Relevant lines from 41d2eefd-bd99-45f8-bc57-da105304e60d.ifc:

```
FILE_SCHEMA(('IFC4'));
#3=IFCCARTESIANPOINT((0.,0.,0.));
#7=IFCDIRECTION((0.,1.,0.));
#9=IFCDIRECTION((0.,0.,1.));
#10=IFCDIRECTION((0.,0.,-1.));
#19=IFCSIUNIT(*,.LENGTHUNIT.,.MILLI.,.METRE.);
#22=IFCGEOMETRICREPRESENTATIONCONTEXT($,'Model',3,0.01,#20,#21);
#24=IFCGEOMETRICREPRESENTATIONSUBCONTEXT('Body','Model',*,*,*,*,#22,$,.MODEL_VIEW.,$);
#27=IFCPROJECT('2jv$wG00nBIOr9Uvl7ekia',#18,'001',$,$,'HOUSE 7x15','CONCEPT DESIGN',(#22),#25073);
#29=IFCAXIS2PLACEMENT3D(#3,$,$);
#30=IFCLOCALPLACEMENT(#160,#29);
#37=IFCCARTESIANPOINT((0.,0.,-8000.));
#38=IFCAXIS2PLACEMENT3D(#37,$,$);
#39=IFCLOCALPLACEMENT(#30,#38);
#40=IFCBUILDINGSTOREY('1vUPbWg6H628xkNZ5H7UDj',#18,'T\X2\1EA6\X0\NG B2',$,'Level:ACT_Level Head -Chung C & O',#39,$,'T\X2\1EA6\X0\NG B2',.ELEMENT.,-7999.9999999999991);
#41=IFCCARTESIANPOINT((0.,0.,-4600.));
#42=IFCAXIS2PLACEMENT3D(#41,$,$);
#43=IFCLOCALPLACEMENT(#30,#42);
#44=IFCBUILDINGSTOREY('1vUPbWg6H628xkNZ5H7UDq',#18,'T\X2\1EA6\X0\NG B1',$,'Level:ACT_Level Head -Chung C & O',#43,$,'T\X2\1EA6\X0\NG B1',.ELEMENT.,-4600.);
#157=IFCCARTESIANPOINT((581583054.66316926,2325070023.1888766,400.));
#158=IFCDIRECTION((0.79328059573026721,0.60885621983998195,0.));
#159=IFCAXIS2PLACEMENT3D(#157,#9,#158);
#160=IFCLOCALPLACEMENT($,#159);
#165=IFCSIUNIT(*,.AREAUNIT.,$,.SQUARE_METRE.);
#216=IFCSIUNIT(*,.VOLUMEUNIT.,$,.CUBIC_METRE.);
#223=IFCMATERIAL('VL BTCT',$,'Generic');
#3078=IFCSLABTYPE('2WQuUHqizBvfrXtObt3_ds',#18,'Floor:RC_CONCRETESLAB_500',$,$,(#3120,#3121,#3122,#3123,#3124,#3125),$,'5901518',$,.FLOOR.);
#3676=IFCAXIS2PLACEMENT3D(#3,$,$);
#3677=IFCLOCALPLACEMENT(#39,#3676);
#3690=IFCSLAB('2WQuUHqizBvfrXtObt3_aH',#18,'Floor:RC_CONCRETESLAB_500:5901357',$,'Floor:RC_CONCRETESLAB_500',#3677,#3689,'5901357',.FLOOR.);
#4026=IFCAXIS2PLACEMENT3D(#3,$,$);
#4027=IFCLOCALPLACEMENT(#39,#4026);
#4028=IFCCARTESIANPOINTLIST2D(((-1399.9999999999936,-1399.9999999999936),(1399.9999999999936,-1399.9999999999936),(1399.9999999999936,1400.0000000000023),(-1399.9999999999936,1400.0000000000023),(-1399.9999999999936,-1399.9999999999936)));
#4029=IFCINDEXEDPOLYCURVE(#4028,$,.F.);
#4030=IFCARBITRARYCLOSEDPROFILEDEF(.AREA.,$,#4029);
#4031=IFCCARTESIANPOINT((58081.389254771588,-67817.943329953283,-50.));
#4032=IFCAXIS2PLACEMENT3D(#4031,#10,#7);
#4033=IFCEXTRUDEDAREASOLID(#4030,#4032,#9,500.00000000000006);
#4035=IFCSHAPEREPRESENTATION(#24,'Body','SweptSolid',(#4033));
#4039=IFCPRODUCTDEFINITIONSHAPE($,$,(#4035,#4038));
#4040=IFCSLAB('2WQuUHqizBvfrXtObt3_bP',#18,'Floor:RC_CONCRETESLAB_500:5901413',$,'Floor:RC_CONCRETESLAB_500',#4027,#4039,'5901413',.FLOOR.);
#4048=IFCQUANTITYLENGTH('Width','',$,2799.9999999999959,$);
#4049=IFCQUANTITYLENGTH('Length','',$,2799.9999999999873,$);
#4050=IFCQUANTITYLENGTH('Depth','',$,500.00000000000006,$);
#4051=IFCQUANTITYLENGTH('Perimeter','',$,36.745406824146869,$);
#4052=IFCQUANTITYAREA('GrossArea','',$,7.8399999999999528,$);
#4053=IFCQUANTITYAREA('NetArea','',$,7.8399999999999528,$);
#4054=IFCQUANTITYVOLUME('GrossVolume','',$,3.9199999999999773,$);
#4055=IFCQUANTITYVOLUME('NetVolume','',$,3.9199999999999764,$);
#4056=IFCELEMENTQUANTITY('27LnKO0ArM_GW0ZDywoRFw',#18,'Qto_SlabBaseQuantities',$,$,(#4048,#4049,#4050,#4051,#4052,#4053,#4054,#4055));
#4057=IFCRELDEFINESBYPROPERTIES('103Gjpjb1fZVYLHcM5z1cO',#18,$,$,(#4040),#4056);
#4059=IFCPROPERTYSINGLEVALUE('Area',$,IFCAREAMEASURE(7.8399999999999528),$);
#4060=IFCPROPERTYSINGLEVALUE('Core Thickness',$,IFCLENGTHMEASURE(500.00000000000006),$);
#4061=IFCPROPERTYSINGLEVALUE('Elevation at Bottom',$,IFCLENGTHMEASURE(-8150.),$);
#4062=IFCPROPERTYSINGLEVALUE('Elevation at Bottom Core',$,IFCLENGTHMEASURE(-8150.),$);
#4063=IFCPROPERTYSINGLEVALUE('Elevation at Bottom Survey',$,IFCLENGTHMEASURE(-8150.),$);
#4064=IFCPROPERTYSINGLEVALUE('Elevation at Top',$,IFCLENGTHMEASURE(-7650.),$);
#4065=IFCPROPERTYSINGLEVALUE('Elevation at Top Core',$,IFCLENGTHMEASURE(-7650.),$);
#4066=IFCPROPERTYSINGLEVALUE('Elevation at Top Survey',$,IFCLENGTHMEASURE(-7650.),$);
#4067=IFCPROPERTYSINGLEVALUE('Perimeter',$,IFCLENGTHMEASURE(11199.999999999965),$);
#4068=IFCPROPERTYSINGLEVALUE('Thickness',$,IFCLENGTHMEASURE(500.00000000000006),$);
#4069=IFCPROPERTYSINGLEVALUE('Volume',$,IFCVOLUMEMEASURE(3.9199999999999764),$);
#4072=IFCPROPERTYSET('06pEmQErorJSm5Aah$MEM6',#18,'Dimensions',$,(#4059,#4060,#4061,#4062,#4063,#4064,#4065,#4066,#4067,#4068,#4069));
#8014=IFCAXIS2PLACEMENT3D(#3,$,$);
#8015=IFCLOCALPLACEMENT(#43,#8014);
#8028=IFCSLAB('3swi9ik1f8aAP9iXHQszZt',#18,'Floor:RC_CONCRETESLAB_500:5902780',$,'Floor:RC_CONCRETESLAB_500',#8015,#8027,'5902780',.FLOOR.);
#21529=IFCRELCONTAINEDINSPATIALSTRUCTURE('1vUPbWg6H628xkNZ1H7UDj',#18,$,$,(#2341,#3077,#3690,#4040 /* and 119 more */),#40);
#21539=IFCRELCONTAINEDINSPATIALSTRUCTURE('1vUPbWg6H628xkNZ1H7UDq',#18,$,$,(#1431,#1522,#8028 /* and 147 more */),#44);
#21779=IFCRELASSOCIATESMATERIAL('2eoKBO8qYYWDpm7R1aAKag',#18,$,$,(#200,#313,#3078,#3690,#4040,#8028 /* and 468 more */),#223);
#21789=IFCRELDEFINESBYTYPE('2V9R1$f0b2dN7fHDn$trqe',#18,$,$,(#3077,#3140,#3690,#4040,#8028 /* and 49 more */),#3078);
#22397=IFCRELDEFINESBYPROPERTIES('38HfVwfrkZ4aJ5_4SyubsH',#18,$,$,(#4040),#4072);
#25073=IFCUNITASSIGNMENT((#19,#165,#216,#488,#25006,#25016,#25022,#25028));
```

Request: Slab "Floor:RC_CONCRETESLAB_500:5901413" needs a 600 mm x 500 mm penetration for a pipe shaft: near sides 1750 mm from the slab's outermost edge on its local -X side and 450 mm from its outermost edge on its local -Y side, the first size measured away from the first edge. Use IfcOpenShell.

```python
import numpy as np
import ifcopenshell
import ifcopenshell.api.feature
import ifcopenshell.api.geometry
import ifcopenshell.api.pset
import ifcopenshell.api.root
import ifcopenshell.geom
import ifcopenshell.util.element
import ifcopenshell.util.placement
import ifcopenshell.util.representation
import ifcopenshell.util.shape
import ifcopenshell.util.unit

model = ifcopenshell.open("41d2eefd-bd99-45f8-bc57-da105304e60d.ifc")
unit_scale = ifcopenshell.util.unit.calculate_unit_scale(model)
area_scale = ifcopenshell.util.unit.calculate_unit_scale(model, "AREAUNIT")
volume_scale = ifcopenshell.util.unit.calculate_unit_scale(model, "VOLUMEUNIT")
settings = ifcopenshell.geom.settings()


def volume(element):
    """Net volume in cubic metres, openings subtracted."""
    shape = ifcopenshell.geom.create_shape(settings, element)
    return ifcopenshell.util.shape.get_volume(shape.geometry)


slab = model.by_id(4040)
before = volume(slab)

# Extent in the slab's own axes, in metres. The edges named are its -X and -Y sides.
slab_shape = ifcopenshell.geom.create_shape(settings, slab)
vertices = ifcopenshell.util.shape.get_vertices(slab_shape.geometry)
x_min, y_min, bottom = vertices.min(axis=0)
top = vertices[:, 2].max()

opening = ifcopenshell.api.root.create_entity(model, ifc_class="IfcOpeningElement", name="Pipe shaft opening", predefined_type="OPENING")
context = ifcopenshell.util.representation.get_context(model, "Model", "Body", "MODEL_VIEW")
width, depth = 0.6, 0.5
outline = [(0.0, 0.0), (width, 0.0), (width, depth), (0.0, depth), (0.0, 0.0)]
# Overshoot both faces by 50 mm so the cut is clean.
shape = ifcopenshell.api.geometry.add_slab_representation(
    model, context=context, depth=top - bottom + 0.1, polyline=outline
)
ifcopenshell.api.geometry.assign_representation(model, product=opening, representation=shape)

matrix = ifcopenshell.util.placement.get_local_placement(slab.ObjectPlacement)
matrix[:, 3] = matrix @ np.append(np.array([x_min + 1.75, y_min + 0.45, bottom - 0.05]) / unit_scale, 1.0)
ifcopenshell.api.geometry.edit_object_placement(model, product=opening, matrix=matrix, is_si=False)
ifcopenshell.api.feature.add_feature(model, feature=opening, element=slab)

after = volume(slab)

# Update the slab's stored quantities.
qto = model.by_id(ifcopenshell.util.element.get_pset(slab, "Qto_SlabBaseQuantities", should_inherit=False)["id"])
ifcopenshell.api.pset.edit_qto(model, qto=qto, properties={
    "NetArea": after / (top - bottom) / area_scale,
    "NetVolume": after / volume_scale,
})
pset = model.by_id(ifcopenshell.util.element.get_pset(slab, "Dimensions", should_inherit=False)["id"])
ifcopenshell.api.pset.edit_pset(model, pset=pset, properties={
    "Area": model.create_entity("IfcAreaMeasure", after / (top - bottom) / area_scale),
    "Volume": model.create_entity("IfcVolumeMeasure", after / volume_scale),
})

print(f"slab volume {before:.3f} -> {after:.3f} m3")

model.write("41d2eefd-bd99-45f8-bc57-da105304e60d_v2.ifc")
```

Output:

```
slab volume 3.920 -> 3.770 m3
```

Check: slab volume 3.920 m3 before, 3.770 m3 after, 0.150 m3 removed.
